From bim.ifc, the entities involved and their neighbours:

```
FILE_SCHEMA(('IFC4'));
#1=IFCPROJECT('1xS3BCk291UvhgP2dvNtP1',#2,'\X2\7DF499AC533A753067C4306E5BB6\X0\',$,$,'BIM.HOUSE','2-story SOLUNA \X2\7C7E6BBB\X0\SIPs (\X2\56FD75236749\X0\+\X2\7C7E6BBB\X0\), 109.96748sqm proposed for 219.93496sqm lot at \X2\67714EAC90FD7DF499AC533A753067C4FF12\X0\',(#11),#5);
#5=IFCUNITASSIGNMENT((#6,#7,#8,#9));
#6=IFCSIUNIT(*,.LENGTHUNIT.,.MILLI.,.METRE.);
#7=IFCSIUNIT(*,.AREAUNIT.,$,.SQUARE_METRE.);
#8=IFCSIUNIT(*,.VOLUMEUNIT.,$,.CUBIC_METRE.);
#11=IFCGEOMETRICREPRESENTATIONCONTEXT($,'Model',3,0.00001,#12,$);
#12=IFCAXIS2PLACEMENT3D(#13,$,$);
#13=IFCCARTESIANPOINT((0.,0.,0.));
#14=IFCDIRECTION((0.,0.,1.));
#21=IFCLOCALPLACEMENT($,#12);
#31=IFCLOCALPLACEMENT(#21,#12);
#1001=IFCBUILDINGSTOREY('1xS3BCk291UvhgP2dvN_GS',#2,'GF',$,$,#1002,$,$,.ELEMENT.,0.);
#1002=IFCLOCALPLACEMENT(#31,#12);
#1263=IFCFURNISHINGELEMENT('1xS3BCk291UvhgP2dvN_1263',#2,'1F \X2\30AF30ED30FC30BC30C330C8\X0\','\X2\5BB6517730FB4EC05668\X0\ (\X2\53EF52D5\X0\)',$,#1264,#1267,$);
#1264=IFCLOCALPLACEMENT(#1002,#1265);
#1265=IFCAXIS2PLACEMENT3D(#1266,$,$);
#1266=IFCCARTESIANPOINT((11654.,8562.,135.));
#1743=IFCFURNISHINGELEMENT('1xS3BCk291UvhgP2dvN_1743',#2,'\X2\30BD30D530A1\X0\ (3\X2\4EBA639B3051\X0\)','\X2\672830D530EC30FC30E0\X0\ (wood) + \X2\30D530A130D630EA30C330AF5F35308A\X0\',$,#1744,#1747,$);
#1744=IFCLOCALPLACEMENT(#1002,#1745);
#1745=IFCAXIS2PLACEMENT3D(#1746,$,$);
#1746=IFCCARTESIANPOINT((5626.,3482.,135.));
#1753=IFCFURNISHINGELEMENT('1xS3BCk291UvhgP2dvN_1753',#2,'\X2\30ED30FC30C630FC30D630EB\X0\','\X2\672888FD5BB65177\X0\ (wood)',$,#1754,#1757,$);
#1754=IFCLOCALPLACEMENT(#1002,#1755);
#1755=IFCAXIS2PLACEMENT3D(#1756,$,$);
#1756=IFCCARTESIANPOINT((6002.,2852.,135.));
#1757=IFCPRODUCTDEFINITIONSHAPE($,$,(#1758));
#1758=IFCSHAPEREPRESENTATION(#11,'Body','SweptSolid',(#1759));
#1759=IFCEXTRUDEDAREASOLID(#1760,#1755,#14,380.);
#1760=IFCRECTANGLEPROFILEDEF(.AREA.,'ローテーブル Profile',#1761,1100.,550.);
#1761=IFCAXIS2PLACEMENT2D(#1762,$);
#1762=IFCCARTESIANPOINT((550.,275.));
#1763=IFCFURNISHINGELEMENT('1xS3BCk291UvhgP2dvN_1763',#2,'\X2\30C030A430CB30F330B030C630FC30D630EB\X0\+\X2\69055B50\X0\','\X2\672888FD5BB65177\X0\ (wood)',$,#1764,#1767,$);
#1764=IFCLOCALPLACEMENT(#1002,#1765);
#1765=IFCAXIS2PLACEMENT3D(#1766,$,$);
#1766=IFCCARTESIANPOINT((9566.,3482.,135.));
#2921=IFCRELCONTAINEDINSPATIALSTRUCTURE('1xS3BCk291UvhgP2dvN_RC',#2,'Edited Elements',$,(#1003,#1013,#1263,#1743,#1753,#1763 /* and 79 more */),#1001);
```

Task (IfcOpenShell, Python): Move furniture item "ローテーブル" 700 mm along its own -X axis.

```python
import ifcopenshell
import ifcopenshell.api.geometry
import ifcopenshell.util.placement
import ifcopenshell.util.unit

model = ifcopenshell.open("bim.ifc")
unit_scale = ifcopenshell.util.unit.calculate_unit_scale(model)

item = model.by_guid("1xS3BCk291UvhgP2dvN_1753")
matrix = ifcopenshell.util.placement.get_local_placement(item.ObjectPlacement)
matrix[:3, 3] -= matrix[:3, 0] * 0.7 / unit_scale
ifcopenshell.api.geometry.edit_object_placement(model, product=item, matrix=matrix, is_si=False)

print(ifcopenshell.util.placement.get_local_placement(item.ObjectPlacement).round(3) + 0.0)

model.write("bim-out.ifc")
```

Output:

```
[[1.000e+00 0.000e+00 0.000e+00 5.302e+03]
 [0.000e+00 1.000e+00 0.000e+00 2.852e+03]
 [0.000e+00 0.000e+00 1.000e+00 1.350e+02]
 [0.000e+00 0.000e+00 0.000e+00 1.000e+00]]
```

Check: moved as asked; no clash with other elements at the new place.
